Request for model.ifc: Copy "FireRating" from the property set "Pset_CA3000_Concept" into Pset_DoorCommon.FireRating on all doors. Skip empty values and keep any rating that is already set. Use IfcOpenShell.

First a look at what the model holds.

```python
import ifcopenshell
import ifcopenshell.util.element

model = ifcopenshell.open("model.ifc")
print(model.schema)
doors = model.by_type("IfcDoor")
print(len(doors), "doors")
for e in doors[:8]:
    source = ifcopenshell.util.element.get_pset(e, "Pset_CA3000_Concept", "FireRating")
    target = ifcopenshell.util.element.get_pset(e, "Pset_DoorCommon", "FireRating")
    print(e.id(), repr(source), repr(target), sep=" | ")
```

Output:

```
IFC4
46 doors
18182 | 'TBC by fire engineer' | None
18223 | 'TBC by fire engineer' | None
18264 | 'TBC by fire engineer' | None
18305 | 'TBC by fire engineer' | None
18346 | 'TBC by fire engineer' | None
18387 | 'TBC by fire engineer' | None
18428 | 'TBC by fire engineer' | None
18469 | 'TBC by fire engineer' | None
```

```python
import ifcopenshell
import ifcopenshell.api.pset
import ifcopenshell.util.element

model = ifcopenshell.open("model.ifc")

count = 0
for e in model.by_type("IfcDoor"):
    value = ifcopenshell.util.element.get_pset(e, "Pset_CA3000_Concept", "FireRating")
    current = ifcopenshell.util.element.get_pset(e, "Pset_DoorCommon", "FireRating")
    if not value or not value.strip() or current:
        continue
    # add_pset returns the element's existing set when there is one.
    pset = ifcopenshell.api.pset.add_pset(model, product=e, name="Pset_DoorCommon")
    ifcopenshell.api.pset.edit_pset(model, pset=pset, properties={"FireRating": value})
    count += 1

print(count, "doors updated")

model.write("model_rev.ifc")
```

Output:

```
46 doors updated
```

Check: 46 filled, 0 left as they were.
